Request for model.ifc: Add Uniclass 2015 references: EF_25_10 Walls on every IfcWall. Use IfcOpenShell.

First a look at what the model holds.

```python
import ifcopenshell

model = ifcopenshell.open("model.ifc")
print(model.schema)
print("classifications:", [c.Name for c in model.by_type("IfcClassification")])
for ifc_class in ("IfcDoor", "IfcRoof", "IfcStair", "IfcWall", "IfcWindow"):
    print(ifc_class, len(model.by_type(ifc_class)))
```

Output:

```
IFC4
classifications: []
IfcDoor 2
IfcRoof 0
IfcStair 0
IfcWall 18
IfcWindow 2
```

```python
import ifcopenshell
import ifcopenshell.api.classification

model = ifcopenshell.open("model.ifc")

system = ifcopenshell.api.classification.add_classification(model, classification="Uniclass 2015")

codes = {
    "IfcWall": ("EF_25_10", "Walls"),
}
for ifc_class, (code, name) in codes.items():
    products = model.by_type(ifc_class)
    ifcopenshell.api.classification.add_reference(
        model, products=products, classification=system, identification=code, name=name
    )
    print(code, len(products))

model.write("model_updated.ifc")
```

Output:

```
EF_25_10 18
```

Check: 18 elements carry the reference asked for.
